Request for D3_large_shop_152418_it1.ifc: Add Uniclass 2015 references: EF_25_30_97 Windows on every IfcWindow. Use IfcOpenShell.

First a look at what the model holds.

```python
import ifcopenshell

model = ifcopenshell.open("D3_large_shop_152418_it1.ifc")
print(model.schema)
print("classifications:", [c.Name for c in model.by_type("IfcClassification")])
for ifc_class in ("IfcDoor", "IfcRoof", "IfcStair", "IfcWall", "IfcWindow"):
    print(ifc_class, len(model.by_type(ifc_class)))
```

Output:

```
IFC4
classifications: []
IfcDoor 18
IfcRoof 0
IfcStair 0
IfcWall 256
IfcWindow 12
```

```python
import ifcopenshell
import ifcopenshell.api.classification

model = ifcopenshell.open("D3_large_shop_152418_it1.ifc")

system = ifcopenshell.api.classification.add_classification(model, classification="Uniclass 2015")

codes = {
    "IfcWindow": ("EF_25_30_97", "Windows"),
}
for ifc_class, (code, name) in codes.items():
    products = model.by_type(ifc_class)
    ifcopenshell.api.classification.add_reference(
        model, products=products, classification=system, identification=code, name=name
    )
    print(code, len(products))

model.write("D3_large_shop_152418_it1_edited.ifc")
```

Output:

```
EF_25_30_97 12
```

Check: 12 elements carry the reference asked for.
